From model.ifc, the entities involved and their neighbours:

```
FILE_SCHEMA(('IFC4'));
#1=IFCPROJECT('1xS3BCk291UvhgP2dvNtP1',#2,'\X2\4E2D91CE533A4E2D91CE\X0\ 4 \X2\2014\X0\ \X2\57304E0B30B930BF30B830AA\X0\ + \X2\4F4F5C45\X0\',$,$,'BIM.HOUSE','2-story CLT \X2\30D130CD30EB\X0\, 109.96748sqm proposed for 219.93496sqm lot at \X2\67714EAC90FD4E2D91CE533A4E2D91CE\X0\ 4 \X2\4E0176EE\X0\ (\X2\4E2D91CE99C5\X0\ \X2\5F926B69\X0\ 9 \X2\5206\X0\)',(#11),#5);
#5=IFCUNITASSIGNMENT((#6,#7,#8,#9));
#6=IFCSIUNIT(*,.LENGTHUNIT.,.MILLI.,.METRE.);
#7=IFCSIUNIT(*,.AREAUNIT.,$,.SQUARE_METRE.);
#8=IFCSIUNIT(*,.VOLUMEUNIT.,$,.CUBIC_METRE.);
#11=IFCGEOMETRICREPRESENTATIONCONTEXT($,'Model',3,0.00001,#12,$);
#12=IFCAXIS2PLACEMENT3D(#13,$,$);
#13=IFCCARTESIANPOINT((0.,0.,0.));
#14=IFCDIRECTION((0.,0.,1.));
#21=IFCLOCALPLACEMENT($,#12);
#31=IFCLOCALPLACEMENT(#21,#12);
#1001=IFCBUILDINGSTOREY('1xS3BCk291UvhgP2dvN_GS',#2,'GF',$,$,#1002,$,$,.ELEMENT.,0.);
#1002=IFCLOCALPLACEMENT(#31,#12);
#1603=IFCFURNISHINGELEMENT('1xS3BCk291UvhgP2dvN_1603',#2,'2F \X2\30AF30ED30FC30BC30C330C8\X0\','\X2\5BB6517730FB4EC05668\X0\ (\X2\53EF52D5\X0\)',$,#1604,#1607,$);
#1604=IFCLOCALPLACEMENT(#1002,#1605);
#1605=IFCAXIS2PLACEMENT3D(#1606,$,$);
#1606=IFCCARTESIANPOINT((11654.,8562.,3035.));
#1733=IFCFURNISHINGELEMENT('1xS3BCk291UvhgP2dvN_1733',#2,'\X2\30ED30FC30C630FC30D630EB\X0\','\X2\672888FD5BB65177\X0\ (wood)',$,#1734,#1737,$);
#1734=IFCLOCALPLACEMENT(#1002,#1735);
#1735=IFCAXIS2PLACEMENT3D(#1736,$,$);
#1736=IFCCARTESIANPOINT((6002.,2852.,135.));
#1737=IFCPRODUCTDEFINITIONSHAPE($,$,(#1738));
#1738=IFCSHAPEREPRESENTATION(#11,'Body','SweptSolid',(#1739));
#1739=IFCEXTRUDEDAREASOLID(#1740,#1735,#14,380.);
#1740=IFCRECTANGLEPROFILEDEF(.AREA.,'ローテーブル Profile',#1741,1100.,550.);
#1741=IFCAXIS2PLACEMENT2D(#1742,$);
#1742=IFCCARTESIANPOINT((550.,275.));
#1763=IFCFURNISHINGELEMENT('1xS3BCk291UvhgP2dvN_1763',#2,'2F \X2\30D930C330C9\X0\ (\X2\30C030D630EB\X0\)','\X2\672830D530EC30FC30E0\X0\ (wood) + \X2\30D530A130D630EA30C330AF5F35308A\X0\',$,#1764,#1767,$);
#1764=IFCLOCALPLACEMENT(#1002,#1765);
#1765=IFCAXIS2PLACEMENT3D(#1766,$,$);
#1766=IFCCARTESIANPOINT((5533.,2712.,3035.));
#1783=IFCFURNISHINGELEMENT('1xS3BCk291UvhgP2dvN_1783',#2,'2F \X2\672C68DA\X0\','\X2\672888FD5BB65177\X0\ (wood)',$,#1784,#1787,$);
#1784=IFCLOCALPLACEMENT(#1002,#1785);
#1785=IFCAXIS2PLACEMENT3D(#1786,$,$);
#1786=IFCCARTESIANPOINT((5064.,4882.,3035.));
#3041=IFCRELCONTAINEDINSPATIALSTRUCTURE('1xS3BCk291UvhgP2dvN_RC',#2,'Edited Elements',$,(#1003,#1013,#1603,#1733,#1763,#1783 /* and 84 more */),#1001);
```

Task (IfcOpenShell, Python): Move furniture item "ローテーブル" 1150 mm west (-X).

```python
import ifcopenshell
import ifcopenshell.api.geometry
import ifcopenshell.util.placement

model = ifcopenshell.open("model.ifc")

item = model.by_guid("1xS3BCk291UvhgP2dvN_1733")
matrix = ifcopenshell.util.placement.get_local_placement(item.ObjectPlacement)
matrix[0, 3] -= 1150.0
ifcopenshell.api.geometry.edit_object_placement(model, product=item, matrix=matrix, is_si=False)

print(ifcopenshell.util.placement.get_local_placement(item.ObjectPlacement).round(3) + 0.0)

model.write("model_edited.ifc")
```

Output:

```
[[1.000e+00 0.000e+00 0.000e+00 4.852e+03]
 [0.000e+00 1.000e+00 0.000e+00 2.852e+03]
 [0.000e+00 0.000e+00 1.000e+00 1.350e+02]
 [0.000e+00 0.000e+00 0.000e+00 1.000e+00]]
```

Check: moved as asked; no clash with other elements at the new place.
